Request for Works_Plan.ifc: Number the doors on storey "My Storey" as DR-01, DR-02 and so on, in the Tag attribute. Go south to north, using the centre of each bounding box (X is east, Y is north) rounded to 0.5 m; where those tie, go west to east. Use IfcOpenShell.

First a look at what the model holds.

```python
import ifcopenshell
import ifcopenshell.util.element
import ifcopenshell.util.placement

model = ifcopenshell.open("Works_Plan.ifc")
print(model.schema)
storey = next(s for s in model.by_type("IfcBuildingStorey") if s.Name == "My Storey")
doors = [e for e in ifcopenshell.util.element.get_decomposition(storey) if e.is_a("IfcDoor")]
for e in sorted(doors, key=lambda e: e.id()):
    origin = ifcopenshell.util.placement.get_local_placement(e.ObjectPlacement)[:3, 3]
    print(e.id(), e.Tag, e.Name, origin.round(2) + 0.0, sep=" | ")
```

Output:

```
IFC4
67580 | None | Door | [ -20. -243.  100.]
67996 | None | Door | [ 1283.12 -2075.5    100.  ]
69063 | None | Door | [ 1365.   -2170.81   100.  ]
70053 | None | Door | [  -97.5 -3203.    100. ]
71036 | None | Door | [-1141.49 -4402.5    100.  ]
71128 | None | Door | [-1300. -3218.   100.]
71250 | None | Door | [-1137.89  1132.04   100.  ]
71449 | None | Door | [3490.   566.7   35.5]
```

```python
import ifcopenshell
import ifcopenshell.geom
import ifcopenshell.util.element
import ifcopenshell.util.shape

model = ifcopenshell.open("Works_Plan.ifc")
settings = ifcopenshell.geom.settings()
settings.set("use-world-coords", True)


def centre(element):
    shape = ifcopenshell.geom.create_shape(settings, element)
    return ifcopenshell.util.shape.get_bbox_centroid(shape.geometry)


storey = next(s for s in model.by_type("IfcBuildingStorey") if s.Name == "My Storey")
doors = [e for e in ifcopenshell.util.element.get_decomposition(storey) if e.is_a("IfcDoor")]

# Insertion points can sit at a corner or the storey origin, so sort by the geometry (in metres).
centres = {e: centre(e) for e in doors}
doors.sort(key=lambda e: (round(centres[e][1] / 0.5), centres[e][0]))

for i, e in enumerate(doors, start=1):
    number = f"DR-{i:02d}"
    e.Tag = number
    print(e.id(), number)

model.write("Works_Plan_edited.ifc")
```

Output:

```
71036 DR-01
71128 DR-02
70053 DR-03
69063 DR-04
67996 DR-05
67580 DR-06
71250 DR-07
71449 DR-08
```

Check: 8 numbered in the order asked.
